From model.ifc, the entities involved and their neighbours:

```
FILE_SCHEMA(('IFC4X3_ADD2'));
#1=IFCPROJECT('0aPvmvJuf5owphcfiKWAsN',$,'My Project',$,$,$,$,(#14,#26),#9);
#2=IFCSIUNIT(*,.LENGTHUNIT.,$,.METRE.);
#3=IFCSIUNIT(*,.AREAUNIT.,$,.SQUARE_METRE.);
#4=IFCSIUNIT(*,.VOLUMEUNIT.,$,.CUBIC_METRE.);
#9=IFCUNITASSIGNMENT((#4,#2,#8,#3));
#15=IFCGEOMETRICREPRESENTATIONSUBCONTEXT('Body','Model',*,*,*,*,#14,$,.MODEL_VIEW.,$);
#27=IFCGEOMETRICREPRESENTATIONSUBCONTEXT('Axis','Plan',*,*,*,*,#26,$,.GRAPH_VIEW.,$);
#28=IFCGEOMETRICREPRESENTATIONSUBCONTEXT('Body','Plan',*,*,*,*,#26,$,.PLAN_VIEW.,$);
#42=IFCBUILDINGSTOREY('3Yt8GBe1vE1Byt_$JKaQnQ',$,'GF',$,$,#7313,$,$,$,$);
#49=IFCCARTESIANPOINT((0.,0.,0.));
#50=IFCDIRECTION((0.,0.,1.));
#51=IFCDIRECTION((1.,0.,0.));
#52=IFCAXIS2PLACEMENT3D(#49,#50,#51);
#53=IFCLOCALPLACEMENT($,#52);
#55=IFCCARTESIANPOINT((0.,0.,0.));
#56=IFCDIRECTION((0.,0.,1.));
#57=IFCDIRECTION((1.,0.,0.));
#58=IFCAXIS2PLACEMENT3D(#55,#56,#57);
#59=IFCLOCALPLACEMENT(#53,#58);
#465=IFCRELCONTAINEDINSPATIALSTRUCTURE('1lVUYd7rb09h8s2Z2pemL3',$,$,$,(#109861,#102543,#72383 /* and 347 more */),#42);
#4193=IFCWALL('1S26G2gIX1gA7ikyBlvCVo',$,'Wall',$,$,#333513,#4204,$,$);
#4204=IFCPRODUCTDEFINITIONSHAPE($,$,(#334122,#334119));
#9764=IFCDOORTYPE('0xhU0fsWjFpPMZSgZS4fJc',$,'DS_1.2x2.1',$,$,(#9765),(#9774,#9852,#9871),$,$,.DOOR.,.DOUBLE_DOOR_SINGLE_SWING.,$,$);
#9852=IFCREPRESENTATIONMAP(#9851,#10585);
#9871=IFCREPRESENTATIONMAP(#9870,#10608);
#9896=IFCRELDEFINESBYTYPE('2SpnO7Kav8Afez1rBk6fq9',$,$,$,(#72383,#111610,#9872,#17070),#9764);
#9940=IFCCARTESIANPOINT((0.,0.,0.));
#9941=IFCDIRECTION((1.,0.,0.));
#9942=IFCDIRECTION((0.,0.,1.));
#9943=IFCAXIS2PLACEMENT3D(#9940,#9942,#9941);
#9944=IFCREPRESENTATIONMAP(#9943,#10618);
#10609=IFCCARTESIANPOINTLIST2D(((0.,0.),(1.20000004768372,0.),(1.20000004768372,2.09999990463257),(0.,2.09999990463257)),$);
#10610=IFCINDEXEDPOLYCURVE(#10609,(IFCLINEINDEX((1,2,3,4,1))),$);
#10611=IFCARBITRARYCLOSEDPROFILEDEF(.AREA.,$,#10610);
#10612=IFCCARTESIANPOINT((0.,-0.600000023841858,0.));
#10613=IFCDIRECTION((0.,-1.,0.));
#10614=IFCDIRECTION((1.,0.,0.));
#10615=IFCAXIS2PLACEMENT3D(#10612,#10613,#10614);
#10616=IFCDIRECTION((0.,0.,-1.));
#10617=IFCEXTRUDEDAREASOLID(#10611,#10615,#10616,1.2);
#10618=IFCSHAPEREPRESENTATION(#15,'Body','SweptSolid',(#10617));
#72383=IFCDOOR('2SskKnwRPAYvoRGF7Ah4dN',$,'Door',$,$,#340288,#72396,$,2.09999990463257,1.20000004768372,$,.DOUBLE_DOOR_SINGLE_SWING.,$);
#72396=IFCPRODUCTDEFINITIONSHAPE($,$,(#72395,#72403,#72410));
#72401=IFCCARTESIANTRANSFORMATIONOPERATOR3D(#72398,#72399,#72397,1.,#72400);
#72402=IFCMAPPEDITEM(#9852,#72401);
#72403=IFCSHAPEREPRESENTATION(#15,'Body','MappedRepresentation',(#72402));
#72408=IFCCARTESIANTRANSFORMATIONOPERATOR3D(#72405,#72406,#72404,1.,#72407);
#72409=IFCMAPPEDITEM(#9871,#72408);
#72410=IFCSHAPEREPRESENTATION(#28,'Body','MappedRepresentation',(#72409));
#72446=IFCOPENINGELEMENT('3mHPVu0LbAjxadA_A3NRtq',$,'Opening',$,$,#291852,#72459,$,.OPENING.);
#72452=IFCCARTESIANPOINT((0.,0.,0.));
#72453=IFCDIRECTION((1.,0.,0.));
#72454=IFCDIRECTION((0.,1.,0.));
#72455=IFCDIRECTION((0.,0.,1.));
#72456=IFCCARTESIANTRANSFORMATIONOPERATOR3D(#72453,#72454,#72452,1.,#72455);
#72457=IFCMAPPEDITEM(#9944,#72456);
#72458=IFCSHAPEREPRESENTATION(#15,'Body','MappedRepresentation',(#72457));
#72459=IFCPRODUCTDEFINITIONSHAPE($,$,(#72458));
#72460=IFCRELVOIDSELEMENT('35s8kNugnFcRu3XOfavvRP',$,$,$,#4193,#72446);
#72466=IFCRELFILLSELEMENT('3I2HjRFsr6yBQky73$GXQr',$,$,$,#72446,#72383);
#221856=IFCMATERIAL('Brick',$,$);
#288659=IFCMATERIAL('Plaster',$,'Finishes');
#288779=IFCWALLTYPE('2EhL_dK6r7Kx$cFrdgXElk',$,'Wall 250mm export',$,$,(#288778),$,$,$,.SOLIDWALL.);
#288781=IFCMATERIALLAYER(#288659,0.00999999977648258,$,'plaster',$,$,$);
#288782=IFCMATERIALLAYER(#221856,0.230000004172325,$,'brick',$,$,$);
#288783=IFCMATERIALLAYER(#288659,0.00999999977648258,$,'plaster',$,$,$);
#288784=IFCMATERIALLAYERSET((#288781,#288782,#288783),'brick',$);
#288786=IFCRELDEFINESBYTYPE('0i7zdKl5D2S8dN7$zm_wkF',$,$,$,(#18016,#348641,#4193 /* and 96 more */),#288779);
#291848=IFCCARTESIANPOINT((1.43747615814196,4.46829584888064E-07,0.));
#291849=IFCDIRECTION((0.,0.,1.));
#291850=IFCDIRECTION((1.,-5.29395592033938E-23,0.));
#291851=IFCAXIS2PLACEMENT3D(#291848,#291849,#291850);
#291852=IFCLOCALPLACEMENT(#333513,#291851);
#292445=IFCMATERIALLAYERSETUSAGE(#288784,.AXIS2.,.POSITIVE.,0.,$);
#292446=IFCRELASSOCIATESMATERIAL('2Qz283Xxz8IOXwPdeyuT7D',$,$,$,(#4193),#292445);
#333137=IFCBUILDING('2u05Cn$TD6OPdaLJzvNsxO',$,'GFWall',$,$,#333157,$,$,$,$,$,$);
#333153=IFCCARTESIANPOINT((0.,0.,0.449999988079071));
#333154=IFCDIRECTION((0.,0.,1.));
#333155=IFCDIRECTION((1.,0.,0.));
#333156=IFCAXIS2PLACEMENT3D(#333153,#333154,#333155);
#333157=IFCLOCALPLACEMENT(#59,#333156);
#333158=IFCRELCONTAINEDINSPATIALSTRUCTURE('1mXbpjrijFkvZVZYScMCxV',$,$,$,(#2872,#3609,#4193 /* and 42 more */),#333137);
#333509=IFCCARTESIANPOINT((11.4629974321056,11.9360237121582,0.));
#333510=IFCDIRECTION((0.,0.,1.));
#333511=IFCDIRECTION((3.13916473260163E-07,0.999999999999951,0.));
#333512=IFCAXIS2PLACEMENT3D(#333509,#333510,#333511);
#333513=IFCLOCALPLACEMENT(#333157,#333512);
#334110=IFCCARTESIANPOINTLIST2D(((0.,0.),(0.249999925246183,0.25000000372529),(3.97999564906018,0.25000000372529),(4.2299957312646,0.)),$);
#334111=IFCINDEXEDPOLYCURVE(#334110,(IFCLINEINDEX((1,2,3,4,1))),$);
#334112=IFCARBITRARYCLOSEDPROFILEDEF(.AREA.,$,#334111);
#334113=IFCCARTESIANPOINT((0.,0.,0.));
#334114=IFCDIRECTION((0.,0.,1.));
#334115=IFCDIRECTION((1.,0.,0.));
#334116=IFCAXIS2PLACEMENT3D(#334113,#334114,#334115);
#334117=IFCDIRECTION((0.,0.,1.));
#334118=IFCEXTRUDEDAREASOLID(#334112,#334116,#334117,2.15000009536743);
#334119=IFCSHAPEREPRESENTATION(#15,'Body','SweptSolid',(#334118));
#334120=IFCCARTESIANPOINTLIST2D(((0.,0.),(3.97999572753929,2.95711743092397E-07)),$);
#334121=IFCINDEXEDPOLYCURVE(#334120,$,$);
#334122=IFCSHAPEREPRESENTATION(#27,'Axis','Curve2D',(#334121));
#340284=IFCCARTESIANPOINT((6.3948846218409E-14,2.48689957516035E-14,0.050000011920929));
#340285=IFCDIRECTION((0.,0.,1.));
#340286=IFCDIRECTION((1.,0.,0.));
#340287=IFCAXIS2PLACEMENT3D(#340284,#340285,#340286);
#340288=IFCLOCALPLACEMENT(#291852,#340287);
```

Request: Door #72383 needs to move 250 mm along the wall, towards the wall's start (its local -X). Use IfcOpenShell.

```python
import ifcopenshell
import ifcopenshell.api.geometry
import ifcopenshell.util.placement
import ifcopenshell.util.unit

model = ifcopenshell.open("model.ifc")
unit_scale = ifcopenshell.util.unit.calculate_unit_scale(model)

door = model.by_guid("2SskKnwRPAYvoRGF7Ah4dN")
opening = door.FillsVoids[0].RelatingOpeningElement
wall = opening.VoidsElements[0].RelatingBuildingElement

wall_matrix = ifcopenshell.util.placement.get_local_placement(wall.ObjectPlacement)
shift = wall_matrix[:3, 0] * -0.25 / unit_scale
before = ifcopenshell.util.placement.get_local_placement(door.ObjectPlacement)[:3, 3].copy()

# The door is placed relative to its opening, so it follows when the opening moves.
matrix = ifcopenshell.util.placement.get_local_placement(opening.ObjectPlacement)
matrix[:3, 3] += shift
ifcopenshell.api.geometry.edit_object_placement(
    model, product=opening, matrix=matrix, is_si=False, should_transform_children=True
)

after = ifcopenshell.util.placement.get_local_placement(door.ObjectPlacement)[:3, 3]
print("door moved by", (after - before).round(3) + 0.0)

model.write("model_updated.ifc")
```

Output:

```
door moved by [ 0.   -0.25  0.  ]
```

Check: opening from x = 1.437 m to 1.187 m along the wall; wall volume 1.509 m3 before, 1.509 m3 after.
